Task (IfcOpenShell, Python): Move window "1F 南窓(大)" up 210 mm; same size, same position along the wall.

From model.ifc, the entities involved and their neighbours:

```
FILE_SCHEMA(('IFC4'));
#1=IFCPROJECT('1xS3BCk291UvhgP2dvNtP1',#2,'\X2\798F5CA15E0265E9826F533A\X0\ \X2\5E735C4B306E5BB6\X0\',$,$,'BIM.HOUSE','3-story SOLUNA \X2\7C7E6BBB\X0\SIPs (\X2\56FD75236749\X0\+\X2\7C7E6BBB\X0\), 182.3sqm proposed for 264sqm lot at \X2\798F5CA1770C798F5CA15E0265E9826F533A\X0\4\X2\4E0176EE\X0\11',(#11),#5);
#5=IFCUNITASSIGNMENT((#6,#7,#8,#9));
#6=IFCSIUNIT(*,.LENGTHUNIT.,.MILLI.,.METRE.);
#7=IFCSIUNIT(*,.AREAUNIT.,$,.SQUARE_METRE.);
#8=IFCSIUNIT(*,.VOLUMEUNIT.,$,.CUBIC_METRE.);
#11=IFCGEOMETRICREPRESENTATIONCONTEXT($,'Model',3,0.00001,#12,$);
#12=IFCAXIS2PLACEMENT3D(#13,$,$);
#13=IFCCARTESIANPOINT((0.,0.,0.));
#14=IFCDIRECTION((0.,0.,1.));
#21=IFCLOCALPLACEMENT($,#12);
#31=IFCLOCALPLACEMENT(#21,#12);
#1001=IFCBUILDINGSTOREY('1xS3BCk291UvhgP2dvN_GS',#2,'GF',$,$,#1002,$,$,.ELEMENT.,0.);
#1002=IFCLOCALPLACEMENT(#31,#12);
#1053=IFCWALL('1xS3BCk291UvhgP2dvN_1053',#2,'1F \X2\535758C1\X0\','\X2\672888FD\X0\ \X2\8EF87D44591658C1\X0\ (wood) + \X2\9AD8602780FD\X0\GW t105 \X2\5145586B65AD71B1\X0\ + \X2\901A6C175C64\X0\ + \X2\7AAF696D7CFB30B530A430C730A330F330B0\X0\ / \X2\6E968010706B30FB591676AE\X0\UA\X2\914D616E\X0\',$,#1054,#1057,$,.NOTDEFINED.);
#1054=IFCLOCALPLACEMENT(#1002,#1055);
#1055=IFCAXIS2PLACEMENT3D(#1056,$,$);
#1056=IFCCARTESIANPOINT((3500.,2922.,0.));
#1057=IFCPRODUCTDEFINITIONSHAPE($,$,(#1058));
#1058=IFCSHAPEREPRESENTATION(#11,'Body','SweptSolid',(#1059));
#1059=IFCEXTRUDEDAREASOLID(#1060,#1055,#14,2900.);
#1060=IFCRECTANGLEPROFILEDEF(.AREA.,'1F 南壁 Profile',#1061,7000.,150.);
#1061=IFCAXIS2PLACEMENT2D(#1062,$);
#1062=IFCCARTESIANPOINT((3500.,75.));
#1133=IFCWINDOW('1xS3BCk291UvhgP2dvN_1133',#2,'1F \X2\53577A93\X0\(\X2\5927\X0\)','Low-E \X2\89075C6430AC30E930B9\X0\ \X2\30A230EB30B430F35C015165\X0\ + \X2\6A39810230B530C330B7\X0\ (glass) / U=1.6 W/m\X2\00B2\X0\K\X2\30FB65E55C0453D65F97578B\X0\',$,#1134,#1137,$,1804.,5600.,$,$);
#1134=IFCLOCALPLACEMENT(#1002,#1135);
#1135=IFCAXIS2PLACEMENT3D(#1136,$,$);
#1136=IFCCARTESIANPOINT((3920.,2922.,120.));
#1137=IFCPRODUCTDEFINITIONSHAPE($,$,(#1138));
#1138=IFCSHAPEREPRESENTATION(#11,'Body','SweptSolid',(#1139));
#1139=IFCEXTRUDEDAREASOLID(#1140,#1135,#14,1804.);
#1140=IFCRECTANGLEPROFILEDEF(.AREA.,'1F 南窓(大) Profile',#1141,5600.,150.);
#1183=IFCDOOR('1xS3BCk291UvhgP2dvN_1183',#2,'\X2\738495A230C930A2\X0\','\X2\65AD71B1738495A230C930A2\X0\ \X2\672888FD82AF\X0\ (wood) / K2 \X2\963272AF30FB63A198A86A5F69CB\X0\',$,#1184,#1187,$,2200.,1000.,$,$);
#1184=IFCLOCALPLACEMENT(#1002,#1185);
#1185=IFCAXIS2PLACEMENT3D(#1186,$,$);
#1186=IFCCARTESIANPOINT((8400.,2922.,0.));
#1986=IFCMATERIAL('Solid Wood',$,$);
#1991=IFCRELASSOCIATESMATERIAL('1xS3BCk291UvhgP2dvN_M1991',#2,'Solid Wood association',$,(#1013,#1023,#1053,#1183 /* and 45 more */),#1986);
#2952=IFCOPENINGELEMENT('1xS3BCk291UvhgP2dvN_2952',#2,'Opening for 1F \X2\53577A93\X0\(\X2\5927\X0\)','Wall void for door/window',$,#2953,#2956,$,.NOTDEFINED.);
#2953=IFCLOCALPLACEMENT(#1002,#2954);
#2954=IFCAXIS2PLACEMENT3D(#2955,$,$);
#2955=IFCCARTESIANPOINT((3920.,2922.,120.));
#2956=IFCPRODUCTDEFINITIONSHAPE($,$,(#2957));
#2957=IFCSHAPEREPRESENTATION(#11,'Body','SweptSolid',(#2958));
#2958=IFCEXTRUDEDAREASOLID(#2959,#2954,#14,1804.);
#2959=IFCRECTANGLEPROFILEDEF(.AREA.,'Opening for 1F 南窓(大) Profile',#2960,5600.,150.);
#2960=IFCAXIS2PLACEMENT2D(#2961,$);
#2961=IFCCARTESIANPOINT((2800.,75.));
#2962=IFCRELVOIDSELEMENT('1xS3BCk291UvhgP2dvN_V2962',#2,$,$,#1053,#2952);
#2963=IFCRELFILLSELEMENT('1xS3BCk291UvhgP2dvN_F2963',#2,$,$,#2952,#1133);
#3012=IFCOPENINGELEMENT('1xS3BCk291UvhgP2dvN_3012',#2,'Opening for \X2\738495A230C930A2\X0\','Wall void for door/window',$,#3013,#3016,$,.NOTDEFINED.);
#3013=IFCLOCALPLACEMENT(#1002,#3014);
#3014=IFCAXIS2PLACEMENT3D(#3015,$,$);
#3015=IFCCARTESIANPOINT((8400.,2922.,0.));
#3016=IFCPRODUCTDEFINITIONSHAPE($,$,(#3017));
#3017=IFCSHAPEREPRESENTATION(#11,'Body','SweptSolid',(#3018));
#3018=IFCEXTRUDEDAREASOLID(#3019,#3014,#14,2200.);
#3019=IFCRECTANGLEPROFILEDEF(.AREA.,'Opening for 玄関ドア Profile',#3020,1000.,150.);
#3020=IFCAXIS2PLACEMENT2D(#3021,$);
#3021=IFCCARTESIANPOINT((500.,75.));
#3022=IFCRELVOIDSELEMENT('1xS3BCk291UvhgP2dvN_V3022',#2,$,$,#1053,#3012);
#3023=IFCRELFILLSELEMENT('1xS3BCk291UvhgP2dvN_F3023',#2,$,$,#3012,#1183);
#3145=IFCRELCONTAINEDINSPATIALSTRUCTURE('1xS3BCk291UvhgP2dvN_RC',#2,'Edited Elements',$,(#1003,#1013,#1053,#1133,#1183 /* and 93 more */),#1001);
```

```python
import numpy as np
import ifcopenshell
import ifcopenshell.api.geometry
import ifcopenshell.util.placement
import ifcopenshell.util.unit

model = ifcopenshell.open("model.ifc")
unit_scale = ifcopenshell.util.unit.calculate_unit_scale(model)

window = model.by_guid("1xS3BCk291UvhgP2dvN_1133")
opening = window.FillsVoids[0].RelatingOpeningElement
dz = 210.0

shift = np.array([0.0, 0.0, dz])
# The window is not placed relative to its opening, so move both.
for product in (opening, window):
    matrix = ifcopenshell.util.placement.get_local_placement(product.ObjectPlacement)
    matrix[:3, 3] += shift
    ifcopenshell.api.geometry.edit_object_placement(model, product=product, matrix=matrix, is_si=False)

print(f"moved by {dz * unit_scale:+.3f} m")

model.write("model_v2.ifc")
```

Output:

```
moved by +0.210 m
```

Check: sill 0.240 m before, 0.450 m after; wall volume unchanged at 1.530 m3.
